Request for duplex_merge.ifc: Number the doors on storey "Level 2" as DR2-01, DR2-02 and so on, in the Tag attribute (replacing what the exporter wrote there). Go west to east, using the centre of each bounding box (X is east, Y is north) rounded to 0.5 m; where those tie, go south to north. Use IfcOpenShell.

First a look at what the model holds.

```python
import ifcopenshell
import ifcopenshell.util.element
import ifcopenshell.util.placement

model = ifcopenshell.open("duplex_merge.ifc")
print(model.schema)
storey = next(s for s in model.by_type("IfcBuildingStorey") if s.Name == "Level 2")
doors = [e for e in ifcopenshell.util.element.get_decomposition(storey) if e.is_a("IfcDoor")]
for e in sorted(doors, key=lambda e: e.id()):
    origin = ifcopenshell.util.placement.get_local_placement(e.ObjectPlacement)[:3, 3]
    print(e.id(), e.Tag, e.Name, origin.round(2) + 0.0, sep=" | ")
```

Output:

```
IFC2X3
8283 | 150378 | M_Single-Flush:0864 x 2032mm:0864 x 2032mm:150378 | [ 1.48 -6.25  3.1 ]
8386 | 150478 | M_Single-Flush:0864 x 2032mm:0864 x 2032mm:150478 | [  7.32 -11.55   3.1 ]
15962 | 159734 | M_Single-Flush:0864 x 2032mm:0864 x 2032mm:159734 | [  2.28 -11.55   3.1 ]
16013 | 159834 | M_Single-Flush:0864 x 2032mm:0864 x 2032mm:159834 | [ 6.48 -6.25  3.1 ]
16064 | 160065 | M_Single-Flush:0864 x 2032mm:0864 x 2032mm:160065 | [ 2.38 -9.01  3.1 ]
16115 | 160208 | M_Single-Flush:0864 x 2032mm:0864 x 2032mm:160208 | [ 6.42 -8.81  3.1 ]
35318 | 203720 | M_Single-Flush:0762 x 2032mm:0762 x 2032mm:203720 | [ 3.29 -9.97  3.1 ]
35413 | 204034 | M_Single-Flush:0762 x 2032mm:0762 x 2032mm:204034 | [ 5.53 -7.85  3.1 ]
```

```python
import ifcopenshell
import ifcopenshell.geom
import ifcopenshell.util.element
import ifcopenshell.util.shape

model = ifcopenshell.open("duplex_merge.ifc")
settings = ifcopenshell.geom.settings()
settings.set("use-world-coords", True)


def centre(element):
    shape = ifcopenshell.geom.create_shape(settings, element)
    return ifcopenshell.util.shape.get_bbox_centroid(shape.geometry)


storey = next(s for s in model.by_type("IfcBuildingStorey") if s.Name == "Level 2")
doors = [e for e in ifcopenshell.util.element.get_decomposition(storey) if e.is_a("IfcDoor")]

# Insertion points can sit at a corner or the storey origin, so sort by the geometry (in metres).
centres = {e: centre(e) for e in doors}
doors.sort(key=lambda e: (round(centres[e][0] / 0.5), centres[e][1]))

for i, e in enumerate(doors, start=1):
    number = f"DR2-{i:02d}"
    e.Tag = number
    print(e.id(), number)

model.write("duplex_merge_edited.ifc")
```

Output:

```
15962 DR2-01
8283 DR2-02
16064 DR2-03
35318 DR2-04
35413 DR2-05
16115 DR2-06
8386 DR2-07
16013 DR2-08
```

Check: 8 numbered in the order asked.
